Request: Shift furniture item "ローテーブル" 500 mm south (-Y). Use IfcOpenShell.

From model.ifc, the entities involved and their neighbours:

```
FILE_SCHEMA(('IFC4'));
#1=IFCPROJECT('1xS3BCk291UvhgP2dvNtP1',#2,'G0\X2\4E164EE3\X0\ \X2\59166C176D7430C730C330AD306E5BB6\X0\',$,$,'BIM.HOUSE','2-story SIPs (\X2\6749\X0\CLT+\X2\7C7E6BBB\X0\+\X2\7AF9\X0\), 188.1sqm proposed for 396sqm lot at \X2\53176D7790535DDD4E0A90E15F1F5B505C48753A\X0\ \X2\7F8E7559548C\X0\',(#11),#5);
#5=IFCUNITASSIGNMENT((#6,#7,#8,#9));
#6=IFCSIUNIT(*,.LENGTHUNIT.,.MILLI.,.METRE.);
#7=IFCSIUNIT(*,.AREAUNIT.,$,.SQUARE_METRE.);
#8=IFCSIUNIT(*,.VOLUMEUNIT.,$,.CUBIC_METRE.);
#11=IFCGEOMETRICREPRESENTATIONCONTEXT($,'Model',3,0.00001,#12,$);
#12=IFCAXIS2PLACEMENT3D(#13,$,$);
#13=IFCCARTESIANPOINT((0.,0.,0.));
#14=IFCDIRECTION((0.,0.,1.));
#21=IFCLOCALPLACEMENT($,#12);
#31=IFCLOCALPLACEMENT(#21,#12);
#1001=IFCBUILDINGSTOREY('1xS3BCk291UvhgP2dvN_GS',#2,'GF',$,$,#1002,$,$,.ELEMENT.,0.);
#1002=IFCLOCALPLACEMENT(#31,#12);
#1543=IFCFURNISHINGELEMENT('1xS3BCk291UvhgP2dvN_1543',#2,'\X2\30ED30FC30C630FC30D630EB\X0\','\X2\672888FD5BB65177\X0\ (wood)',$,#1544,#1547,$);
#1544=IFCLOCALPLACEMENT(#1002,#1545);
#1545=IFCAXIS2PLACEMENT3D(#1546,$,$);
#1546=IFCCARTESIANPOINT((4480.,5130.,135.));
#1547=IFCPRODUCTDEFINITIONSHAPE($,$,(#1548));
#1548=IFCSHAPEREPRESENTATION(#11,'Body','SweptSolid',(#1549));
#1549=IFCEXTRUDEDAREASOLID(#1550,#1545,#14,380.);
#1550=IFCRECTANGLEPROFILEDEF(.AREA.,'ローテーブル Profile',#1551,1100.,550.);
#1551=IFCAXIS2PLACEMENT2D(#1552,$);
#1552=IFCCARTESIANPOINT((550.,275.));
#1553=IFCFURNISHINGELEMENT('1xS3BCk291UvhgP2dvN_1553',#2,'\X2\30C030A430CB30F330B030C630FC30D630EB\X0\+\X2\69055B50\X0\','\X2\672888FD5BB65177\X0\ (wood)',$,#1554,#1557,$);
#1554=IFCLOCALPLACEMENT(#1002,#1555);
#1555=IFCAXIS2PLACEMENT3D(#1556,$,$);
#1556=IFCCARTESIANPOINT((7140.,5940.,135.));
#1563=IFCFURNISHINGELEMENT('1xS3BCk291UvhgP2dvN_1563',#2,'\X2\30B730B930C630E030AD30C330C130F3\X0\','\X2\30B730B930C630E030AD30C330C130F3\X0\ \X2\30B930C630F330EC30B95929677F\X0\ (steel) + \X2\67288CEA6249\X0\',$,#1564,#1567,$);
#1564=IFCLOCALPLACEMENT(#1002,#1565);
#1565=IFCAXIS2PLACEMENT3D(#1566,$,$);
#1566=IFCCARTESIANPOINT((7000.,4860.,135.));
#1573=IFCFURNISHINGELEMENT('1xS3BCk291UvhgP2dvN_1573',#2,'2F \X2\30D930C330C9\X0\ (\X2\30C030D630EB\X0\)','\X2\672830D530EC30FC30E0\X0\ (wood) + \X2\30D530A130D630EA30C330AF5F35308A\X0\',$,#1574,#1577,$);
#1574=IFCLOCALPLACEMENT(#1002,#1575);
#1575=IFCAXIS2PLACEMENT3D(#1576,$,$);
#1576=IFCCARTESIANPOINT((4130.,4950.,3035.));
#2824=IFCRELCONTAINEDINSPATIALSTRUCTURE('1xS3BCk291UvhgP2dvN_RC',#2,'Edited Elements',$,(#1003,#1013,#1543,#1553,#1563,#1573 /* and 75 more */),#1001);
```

```python
import ifcopenshell
import ifcopenshell.api.geometry
import ifcopenshell.util.placement
import ifcopenshell.util.unit

model = ifcopenshell.open("model.ifc")
unit_scale = ifcopenshell.util.unit.calculate_unit_scale(model)

item = model.by_id(1543)
matrix = ifcopenshell.util.placement.get_local_placement(item.ObjectPlacement)
matrix[1, 3] -= 0.5 / unit_scale
ifcopenshell.api.geometry.edit_object_placement(model, product=item, matrix=matrix, is_si=False)

print(ifcopenshell.util.placement.get_local_placement(item.ObjectPlacement).round(3) + 0.0)

model.write("model_edited.ifc")
```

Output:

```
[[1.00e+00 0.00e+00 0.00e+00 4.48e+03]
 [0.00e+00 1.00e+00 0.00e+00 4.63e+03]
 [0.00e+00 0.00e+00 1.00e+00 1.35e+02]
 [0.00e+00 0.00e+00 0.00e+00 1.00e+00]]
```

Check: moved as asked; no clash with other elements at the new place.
